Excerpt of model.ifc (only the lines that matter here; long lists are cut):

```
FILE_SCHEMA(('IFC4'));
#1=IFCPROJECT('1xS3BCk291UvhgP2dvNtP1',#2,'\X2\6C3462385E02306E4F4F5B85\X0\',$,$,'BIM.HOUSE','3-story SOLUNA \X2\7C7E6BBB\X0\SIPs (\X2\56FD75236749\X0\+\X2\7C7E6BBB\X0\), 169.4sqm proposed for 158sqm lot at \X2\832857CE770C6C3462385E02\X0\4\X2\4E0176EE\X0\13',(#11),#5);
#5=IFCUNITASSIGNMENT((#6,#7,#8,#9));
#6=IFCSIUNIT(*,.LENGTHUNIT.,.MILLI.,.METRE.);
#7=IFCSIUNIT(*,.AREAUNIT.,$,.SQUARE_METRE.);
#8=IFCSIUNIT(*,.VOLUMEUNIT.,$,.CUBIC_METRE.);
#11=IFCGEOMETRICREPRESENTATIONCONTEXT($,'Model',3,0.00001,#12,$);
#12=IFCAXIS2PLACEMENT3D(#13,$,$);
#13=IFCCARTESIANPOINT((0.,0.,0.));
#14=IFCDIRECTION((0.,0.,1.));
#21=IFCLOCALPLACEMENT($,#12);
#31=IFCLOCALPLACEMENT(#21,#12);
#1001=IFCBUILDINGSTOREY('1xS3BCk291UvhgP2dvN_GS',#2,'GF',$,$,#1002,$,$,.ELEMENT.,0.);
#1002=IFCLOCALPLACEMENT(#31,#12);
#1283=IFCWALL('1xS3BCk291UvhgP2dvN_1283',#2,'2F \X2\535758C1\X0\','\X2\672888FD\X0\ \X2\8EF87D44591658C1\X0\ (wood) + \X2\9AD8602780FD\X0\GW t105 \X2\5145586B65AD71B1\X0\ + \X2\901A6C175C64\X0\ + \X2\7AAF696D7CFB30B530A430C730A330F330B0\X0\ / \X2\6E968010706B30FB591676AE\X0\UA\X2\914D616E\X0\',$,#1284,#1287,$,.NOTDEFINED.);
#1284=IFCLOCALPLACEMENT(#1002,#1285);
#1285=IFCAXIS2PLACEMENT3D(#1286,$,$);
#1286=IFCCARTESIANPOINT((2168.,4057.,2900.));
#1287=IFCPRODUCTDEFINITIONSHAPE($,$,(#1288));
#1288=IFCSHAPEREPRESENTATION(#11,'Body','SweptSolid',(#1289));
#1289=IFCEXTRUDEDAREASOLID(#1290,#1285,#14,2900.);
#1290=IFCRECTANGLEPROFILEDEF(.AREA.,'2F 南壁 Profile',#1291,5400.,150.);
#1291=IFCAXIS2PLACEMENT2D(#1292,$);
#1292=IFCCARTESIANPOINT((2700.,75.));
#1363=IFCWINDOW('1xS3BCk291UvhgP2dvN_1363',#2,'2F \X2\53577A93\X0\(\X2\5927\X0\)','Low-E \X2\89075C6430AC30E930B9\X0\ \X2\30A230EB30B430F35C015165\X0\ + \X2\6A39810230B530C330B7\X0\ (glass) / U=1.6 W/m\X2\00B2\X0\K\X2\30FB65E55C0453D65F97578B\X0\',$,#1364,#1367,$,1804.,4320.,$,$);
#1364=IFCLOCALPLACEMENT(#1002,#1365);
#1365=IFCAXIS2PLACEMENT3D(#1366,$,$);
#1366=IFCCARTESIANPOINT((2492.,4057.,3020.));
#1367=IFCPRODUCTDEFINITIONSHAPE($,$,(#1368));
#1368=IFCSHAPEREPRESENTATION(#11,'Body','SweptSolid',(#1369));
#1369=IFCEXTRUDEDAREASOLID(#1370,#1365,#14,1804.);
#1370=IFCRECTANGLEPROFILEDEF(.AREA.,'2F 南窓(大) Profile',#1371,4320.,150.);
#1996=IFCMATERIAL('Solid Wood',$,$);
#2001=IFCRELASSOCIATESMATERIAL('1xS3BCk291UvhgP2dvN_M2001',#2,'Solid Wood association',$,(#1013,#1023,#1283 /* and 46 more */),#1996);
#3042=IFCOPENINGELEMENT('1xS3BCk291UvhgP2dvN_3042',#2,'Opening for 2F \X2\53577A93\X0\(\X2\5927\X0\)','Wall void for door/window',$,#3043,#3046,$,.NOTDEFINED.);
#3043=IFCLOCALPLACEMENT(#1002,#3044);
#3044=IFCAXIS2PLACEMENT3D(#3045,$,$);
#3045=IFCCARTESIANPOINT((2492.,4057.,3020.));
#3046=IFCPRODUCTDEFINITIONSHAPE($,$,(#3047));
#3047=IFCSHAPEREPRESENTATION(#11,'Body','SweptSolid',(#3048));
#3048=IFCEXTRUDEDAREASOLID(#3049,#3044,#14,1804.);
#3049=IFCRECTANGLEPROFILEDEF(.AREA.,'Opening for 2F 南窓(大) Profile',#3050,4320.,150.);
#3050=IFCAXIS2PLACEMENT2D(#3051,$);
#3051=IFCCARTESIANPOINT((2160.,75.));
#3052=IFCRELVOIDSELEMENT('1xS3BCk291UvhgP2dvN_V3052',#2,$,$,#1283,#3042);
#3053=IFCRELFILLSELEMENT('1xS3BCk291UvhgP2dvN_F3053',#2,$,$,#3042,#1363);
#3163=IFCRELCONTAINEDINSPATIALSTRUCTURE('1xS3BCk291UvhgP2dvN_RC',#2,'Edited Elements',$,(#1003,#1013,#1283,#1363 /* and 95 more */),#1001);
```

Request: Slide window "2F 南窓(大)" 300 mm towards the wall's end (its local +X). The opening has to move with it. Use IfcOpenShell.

```python
import ifcopenshell
import ifcopenshell.api.geometry
import ifcopenshell.util.placement

model = ifcopenshell.open("model.ifc")

window = model.by_id(1363)
opening = window.FillsVoids[0].RelatingOpeningElement
wall = opening.VoidsElements[0].RelatingBuildingElement

wall_matrix = ifcopenshell.util.placement.get_local_placement(wall.ObjectPlacement)
shift = wall_matrix[:3, 0] * 300.0
before = ifcopenshell.util.placement.get_local_placement(window.ObjectPlacement)[:3, 3].copy()

# The window is not placed relative to its opening, so move both.
for product in (opening, window):
    matrix = ifcopenshell.util.placement.get_local_placement(product.ObjectPlacement)
    matrix[:3, 3] += shift
    ifcopenshell.api.geometry.edit_object_placement(model, product=product, matrix=matrix, is_si=False)

after = ifcopenshell.util.placement.get_local_placement(window.ObjectPlacement)[:3, 3]
print("window moved by", (after - before).round(3) + 0.0)

model.write("model_rev.ifc")
```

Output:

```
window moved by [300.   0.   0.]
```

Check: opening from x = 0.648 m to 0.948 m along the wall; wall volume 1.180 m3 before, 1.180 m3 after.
